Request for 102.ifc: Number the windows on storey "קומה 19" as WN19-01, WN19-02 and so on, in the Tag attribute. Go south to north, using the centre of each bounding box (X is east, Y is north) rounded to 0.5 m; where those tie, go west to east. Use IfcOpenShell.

First a look at what the model holds.

```python
import ifcopenshell
import ifcopenshell.util.element
import ifcopenshell.util.placement

model = ifcopenshell.open("102.ifc")
print(model.schema)
storey = next(s for s in model.by_type("IfcBuildingStorey") if s.Name == "קומה 19")
windows = [e for e in ifcopenshell.util.element.get_decomposition(storey) if e.is_a("IfcWindow")]
for e in sorted(windows, key=lambda e: e.id()):
    origin = ifcopenshell.util.placement.get_local_placement(e.ObjectPlacement)[:3, 3]
    print(e.id(), e.Tag, e.Name, origin.round(2) + 0.0, sep=" | ")
```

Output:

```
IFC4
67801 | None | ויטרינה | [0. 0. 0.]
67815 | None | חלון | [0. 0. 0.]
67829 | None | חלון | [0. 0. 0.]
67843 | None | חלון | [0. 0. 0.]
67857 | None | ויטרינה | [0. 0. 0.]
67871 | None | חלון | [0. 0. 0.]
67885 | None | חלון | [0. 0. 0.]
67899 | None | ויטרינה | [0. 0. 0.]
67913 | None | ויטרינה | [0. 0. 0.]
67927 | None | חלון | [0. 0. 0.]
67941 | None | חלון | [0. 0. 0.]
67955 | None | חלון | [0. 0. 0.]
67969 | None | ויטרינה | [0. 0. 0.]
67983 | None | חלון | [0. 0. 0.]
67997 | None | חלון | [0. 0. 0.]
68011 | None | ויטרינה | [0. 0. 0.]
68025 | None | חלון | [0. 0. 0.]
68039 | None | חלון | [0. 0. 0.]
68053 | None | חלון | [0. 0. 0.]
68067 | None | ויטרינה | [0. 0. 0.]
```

```python
import ifcopenshell
import ifcopenshell.geom
import ifcopenshell.util.element
import ifcopenshell.util.shape

model = ifcopenshell.open("102.ifc")
settings = ifcopenshell.geom.settings()
settings.set("use-world-coords", True)


def centre(element):
    shape = ifcopenshell.geom.create_shape(settings, element)
    return ifcopenshell.util.shape.get_bbox_centroid(shape.geometry)


storey = next(s for s in model.by_type("IfcBuildingStorey") if s.Name == "קומה 19")
windows = [e for e in ifcopenshell.util.element.get_decomposition(storey) if e.is_a("IfcWindow")]

# Insertion points can sit at a corner or the storey origin, so sort by the geometry (in metres).
centres = {e: centre(e) for e in windows}
windows.sort(key=lambda e: (round(centres[e][1] / 0.5), centres[e][0]))

for i, e in enumerate(windows, start=1):
    number = f"WN19-{i:02d}"
    e.Tag = number
    print(e.id(), number)

model.write("102_edited.ifc")
```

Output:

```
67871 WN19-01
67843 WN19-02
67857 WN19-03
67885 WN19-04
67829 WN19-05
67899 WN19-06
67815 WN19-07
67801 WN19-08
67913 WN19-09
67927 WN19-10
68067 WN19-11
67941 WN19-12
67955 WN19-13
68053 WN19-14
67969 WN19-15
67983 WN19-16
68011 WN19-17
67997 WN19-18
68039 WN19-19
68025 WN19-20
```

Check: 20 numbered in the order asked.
